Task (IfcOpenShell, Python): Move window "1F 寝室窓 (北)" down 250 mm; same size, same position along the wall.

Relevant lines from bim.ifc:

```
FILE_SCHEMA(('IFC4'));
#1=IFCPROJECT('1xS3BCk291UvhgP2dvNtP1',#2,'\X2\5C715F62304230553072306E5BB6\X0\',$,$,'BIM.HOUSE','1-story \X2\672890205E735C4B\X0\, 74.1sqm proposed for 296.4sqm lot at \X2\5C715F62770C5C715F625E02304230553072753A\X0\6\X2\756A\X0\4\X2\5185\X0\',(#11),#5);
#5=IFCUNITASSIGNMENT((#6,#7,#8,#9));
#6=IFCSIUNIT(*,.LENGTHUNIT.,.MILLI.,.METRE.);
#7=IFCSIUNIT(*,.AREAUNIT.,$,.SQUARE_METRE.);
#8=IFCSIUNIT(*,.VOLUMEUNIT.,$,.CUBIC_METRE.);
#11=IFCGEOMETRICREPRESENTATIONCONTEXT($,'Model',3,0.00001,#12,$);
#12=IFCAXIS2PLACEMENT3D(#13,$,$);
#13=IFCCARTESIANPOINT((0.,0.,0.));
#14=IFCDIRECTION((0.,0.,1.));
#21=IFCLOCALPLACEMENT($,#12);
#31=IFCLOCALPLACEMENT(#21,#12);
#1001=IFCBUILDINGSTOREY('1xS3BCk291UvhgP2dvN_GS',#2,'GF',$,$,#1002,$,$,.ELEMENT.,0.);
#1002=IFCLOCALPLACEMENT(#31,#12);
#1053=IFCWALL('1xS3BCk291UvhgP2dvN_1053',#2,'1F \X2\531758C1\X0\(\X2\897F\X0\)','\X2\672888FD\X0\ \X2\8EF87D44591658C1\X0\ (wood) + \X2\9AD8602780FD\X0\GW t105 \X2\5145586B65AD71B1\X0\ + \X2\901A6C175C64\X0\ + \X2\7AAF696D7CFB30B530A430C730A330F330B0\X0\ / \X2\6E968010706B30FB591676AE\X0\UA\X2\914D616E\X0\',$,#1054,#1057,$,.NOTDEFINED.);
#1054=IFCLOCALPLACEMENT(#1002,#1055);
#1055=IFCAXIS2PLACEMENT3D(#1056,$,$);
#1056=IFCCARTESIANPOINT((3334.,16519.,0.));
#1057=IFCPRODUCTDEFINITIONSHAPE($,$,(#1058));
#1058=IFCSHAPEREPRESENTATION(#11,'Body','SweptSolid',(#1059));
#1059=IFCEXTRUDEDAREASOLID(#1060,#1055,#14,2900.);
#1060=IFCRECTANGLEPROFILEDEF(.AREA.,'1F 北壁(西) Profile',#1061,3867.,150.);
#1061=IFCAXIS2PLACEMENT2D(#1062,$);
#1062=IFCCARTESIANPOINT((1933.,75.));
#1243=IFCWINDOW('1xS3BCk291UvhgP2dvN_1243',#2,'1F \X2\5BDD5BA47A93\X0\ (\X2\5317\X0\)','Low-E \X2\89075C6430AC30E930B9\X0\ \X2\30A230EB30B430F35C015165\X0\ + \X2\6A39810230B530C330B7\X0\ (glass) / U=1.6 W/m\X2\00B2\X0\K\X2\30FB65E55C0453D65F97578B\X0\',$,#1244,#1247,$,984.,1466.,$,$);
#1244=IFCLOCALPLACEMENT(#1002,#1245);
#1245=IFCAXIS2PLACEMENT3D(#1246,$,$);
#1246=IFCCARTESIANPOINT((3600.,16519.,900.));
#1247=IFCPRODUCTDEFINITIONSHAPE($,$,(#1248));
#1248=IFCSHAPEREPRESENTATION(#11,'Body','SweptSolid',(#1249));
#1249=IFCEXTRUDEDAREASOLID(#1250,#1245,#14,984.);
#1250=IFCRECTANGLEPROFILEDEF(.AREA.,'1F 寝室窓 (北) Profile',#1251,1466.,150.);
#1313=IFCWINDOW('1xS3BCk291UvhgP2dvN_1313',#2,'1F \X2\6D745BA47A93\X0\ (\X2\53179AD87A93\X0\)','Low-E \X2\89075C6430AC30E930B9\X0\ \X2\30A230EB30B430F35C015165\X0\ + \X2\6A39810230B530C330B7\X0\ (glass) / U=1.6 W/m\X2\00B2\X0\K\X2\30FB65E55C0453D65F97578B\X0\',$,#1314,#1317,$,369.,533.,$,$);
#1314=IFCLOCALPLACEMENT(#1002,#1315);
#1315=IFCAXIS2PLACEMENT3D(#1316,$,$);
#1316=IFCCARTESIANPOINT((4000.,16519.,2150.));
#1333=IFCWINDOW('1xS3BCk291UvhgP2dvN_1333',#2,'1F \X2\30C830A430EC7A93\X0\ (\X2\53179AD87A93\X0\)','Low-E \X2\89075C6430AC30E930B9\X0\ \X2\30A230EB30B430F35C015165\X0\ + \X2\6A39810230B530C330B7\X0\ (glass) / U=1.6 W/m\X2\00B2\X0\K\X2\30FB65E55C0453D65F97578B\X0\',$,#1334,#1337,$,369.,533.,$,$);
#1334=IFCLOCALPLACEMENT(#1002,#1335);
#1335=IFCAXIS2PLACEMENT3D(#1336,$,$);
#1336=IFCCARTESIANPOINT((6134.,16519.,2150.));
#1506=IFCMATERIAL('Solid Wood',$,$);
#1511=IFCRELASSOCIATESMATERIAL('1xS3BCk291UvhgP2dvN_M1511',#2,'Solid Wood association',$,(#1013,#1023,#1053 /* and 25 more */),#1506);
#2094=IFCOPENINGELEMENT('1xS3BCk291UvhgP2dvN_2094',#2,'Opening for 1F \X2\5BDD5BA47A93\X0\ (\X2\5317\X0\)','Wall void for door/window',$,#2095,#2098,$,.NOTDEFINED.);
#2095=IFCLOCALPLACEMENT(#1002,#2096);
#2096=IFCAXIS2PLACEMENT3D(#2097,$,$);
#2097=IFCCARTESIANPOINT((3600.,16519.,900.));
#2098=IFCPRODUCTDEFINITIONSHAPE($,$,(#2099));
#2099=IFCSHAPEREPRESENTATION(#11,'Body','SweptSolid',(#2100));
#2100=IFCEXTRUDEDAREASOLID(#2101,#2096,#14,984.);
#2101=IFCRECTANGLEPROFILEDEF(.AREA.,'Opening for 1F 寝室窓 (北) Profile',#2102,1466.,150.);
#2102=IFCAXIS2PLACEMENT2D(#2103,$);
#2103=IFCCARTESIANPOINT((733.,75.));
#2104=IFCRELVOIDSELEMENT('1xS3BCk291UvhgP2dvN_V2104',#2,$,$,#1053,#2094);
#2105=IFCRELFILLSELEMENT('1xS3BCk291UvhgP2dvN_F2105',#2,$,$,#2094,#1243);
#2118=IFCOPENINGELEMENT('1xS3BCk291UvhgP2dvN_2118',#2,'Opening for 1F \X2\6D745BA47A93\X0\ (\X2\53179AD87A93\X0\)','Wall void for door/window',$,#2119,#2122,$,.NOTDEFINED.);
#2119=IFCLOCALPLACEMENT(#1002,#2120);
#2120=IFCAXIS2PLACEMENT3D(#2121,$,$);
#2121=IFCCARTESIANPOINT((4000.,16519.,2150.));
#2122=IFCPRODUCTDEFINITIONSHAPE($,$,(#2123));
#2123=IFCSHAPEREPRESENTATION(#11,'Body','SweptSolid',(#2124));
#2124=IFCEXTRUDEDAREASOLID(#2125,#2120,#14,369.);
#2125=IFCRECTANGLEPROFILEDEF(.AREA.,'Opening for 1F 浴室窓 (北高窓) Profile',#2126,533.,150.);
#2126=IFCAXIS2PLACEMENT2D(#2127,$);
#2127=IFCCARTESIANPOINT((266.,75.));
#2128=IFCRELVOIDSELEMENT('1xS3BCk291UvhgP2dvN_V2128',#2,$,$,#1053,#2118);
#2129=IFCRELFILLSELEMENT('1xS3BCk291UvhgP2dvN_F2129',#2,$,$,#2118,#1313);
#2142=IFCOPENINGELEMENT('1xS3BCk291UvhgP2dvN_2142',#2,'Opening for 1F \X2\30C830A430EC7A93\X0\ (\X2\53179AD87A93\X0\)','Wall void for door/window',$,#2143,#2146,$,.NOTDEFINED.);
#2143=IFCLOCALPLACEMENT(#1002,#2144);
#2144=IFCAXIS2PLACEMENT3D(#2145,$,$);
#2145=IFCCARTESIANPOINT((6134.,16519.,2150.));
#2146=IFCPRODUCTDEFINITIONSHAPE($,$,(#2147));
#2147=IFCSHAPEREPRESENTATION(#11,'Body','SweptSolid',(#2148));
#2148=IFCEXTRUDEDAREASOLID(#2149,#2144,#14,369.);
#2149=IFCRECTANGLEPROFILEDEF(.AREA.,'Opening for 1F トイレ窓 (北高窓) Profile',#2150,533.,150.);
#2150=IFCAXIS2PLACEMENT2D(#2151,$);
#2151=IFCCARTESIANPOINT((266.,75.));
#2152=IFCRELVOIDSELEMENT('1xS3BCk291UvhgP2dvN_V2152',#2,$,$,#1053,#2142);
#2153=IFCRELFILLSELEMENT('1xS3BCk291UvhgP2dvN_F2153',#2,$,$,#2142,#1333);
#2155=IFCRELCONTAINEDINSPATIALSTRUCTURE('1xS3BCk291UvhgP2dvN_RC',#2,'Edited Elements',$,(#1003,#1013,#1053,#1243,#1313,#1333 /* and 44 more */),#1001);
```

```python
import numpy as np
import ifcopenshell
import ifcopenshell.api.geometry
import ifcopenshell.util.placement
import ifcopenshell.util.unit

model = ifcopenshell.open("bim.ifc")
unit_scale = ifcopenshell.util.unit.calculate_unit_scale(model)

window = model.by_guid("1xS3BCk291UvhgP2dvN_1243")
opening = window.FillsVoids[0].RelatingOpeningElement
dz = -250.0

shift = np.array([0.0, 0.0, dz])
# The window is not placed relative to its opening, so move both.
for product in (opening, window):
    matrix = ifcopenshell.util.placement.get_local_placement(product.ObjectPlacement)
    matrix[:3, 3] += shift
    ifcopenshell.api.geometry.edit_object_placement(model, product=product, matrix=matrix, is_si=False)

print(f"moved by {dz * unit_scale:+.3f} m")

model.write("bim_updated.ifc")
```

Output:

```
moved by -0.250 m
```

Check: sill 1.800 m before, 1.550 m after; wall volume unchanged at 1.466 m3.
